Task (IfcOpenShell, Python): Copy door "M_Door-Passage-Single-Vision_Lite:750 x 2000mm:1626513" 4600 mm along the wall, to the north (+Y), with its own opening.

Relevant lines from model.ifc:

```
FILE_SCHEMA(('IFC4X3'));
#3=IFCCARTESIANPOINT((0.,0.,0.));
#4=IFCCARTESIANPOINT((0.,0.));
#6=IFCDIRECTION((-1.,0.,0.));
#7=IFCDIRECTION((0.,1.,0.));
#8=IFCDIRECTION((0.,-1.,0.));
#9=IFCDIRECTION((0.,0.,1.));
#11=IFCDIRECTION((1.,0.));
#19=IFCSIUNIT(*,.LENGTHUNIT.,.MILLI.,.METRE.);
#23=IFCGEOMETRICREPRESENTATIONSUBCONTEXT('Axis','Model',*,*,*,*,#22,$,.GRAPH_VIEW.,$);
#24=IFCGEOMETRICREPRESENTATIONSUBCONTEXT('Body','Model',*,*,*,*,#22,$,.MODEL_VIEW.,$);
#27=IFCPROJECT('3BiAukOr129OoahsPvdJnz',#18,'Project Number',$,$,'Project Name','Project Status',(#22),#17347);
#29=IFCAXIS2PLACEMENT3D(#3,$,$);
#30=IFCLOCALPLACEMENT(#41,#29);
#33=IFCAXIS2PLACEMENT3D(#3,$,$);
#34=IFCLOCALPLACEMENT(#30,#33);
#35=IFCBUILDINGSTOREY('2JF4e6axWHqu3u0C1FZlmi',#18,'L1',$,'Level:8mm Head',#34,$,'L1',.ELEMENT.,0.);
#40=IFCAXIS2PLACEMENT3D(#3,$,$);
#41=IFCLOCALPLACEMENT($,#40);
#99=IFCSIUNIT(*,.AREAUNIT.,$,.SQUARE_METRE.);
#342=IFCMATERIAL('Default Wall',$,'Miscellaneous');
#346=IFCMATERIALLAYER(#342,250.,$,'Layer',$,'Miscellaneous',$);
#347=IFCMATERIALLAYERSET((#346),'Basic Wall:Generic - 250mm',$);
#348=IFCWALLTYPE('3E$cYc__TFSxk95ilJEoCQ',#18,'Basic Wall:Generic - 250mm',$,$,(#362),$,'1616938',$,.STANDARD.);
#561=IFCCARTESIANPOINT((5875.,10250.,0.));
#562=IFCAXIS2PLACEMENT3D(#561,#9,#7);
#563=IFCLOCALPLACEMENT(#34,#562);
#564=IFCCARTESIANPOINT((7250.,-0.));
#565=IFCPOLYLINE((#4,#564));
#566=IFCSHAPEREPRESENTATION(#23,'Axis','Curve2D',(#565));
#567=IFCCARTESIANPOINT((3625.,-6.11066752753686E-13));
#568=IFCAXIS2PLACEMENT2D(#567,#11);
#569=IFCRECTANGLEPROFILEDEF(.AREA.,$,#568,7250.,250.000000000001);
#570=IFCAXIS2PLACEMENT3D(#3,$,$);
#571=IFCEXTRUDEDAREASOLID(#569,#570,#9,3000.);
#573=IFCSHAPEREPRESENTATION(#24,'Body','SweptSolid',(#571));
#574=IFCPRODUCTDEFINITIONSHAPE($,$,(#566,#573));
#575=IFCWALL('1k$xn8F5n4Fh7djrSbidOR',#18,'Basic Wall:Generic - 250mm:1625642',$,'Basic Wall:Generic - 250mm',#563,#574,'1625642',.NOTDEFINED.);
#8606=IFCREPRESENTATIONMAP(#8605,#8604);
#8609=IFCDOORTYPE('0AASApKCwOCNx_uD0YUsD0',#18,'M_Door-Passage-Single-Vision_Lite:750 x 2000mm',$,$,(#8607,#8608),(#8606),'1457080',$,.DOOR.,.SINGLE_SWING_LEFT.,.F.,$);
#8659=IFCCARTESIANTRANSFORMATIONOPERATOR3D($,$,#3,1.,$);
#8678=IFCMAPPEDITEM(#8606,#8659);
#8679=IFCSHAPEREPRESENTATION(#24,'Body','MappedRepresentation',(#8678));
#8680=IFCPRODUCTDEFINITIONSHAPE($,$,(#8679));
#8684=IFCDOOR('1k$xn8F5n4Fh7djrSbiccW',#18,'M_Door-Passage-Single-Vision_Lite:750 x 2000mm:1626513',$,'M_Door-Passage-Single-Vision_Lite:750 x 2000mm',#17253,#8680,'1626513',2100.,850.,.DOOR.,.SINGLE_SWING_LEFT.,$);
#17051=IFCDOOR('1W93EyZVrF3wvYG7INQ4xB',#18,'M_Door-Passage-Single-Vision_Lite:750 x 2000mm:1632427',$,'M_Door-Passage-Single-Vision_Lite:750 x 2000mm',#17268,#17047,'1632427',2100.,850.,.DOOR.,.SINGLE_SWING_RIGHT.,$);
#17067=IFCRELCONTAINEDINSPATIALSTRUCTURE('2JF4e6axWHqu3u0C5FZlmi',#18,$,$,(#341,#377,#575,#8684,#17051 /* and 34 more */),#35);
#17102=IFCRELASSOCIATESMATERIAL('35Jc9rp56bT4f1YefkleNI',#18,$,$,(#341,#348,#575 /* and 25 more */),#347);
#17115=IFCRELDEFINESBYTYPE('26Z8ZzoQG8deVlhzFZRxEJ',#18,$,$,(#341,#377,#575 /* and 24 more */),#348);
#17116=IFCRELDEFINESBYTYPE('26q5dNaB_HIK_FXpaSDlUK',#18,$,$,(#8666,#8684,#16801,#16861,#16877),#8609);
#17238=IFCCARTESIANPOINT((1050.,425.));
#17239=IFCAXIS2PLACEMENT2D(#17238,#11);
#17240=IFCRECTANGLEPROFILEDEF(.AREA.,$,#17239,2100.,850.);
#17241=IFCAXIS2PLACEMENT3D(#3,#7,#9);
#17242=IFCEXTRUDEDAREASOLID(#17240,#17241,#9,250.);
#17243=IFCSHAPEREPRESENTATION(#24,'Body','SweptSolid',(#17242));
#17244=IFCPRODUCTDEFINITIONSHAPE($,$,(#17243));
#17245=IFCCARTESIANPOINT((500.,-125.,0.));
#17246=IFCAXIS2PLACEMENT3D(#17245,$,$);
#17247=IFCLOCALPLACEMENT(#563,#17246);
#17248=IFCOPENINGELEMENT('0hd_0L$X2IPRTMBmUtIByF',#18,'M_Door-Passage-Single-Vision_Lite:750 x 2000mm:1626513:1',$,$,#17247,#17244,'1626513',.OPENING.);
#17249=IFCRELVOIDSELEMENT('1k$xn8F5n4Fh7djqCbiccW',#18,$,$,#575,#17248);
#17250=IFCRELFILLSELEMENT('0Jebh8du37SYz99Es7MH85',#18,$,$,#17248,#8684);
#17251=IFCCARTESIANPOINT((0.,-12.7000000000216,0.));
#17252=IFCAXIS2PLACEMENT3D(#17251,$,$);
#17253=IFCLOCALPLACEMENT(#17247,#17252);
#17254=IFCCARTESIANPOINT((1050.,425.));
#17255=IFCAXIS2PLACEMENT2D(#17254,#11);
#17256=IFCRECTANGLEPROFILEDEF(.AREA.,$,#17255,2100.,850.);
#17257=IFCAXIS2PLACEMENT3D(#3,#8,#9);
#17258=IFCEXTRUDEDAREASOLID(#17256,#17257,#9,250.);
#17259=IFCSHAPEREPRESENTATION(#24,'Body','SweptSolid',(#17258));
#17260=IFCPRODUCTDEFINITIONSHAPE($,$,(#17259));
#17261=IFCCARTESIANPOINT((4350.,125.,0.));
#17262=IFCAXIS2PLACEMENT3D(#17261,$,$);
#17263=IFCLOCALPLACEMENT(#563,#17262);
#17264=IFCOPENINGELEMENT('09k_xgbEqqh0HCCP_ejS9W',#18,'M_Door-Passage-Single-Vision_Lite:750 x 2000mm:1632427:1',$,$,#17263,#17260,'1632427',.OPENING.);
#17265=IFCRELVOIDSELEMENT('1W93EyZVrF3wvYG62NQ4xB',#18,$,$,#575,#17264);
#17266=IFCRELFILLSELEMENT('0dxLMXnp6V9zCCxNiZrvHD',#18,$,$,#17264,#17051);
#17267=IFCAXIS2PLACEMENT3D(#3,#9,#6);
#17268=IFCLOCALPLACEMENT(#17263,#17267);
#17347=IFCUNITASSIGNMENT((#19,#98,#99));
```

```python
import ifcopenshell
import ifcopenshell.api.feature
import ifcopenshell.api.geometry
import ifcopenshell.api.root
import ifcopenshell.geom
import ifcopenshell.util.element
import ifcopenshell.util.placement
import ifcopenshell.util.shape

model = ifcopenshell.open("model.ifc")
settings = ifcopenshell.geom.settings()


def volume(element):
    """Net volume in cubic metres, openings subtracted."""
    shape = ifcopenshell.geom.create_shape(settings, element)
    return ifcopenshell.util.shape.get_volume(shape.geometry)


def reuse_history(source, copy):
    """copy_class also copies each property set's owner history, people and application; keep the originals."""
    for rel in copy.IsDefinedBy:
        if rel.is_a("IfcRelDefinesByProperties") and (history := rel.RelatingPropertyDefinition.OwnerHistory):
            rel.RelatingPropertyDefinition.OwnerHistory = source.OwnerHistory
            ifcopenshell.util.element.remove_deep2(model, history)


door = model.by_id(8684)
opening = door.FillsVoids[0].RelatingOpeningElement
wall = opening.VoidsElements[0].RelatingBuildingElement
before = volume(wall)
shift = ifcopenshell.util.placement.get_local_placement(wall.ObjectPlacement)[:3, 0] * 4600.0

# copy_class copies the void relationship, type, container and properties, but no geometry.
new_opening = ifcopenshell.api.root.copy_class(model, product=opening)
new_opening.Representation = ifcopenshell.util.element.copy_deep(
    model, opening.Representation, exclude=["IfcGeometricRepresentationContext", "IfcRepresentationMap"]
)
new_opening.Name = "M_Door-Passage-Single-Vision_Lite:750 x 2000mm"
new_opening.Tag = None
new_door = ifcopenshell.api.root.copy_class(model, product=door)
new_door.Representation = ifcopenshell.util.element.copy_deep(
    model, door.Representation, exclude=["IfcGeometricRepresentationContext", "IfcRepresentationMap"]
)
new_door.Name = "M_Door-Passage-Single-Vision_Lite:750 x 2000mm"
new_door.Tag = None
reuse_history(door, new_door)
ifcopenshell.api.feature.add_filling(model, opening=new_opening, element=new_door)

for old, new in ((opening, new_opening), (door, new_door)):
    matrix = ifcopenshell.util.placement.get_local_placement(old.ObjectPlacement)
    matrix[:3, 3] += shift
    ifcopenshell.api.geometry.edit_object_placement(model, product=new, matrix=matrix, is_si=False)

after = volume(wall)

print(f"wall volume {before:.3f} -> {after:.3f} m3")

model.write("model_edited.ifc")
```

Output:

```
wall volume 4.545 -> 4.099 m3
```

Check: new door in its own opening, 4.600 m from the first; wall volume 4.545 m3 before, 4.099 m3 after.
